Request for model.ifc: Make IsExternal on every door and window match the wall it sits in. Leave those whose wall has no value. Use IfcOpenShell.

First a look at what the model holds.

```python
import ifcopenshell
import ifcopenshell.util.element

model = ifcopenshell.open("model.ifc")
print(model.schema)
seen = {}
for e in model.by_type("IfcDoor") + model.by_type("IfcWindow"):
    if not e.FillsVoids:
        continue
    host = e.FillsVoids[0].RelatingOpeningElement.VoidsElements[0].RelatingBuildingElement
    own = ifcopenshell.util.element.get_pset(e, f"Pset_{e.is_a()[3:].removesuffix('StandardCase')}Common", "IsExternal")
    wall = ifcopenshell.util.element.get_pset(host, "Pset_WallCommon", "IsExternal")
    seen[e.is_a(), own, wall] = seen.get((e.is_a(), own, wall), 0) + 1
for (cls, own, wall), count in sorted(seen.items(), key=str):
    print(count, cls, "IsExternal:", own, "| host wall:", wall)
```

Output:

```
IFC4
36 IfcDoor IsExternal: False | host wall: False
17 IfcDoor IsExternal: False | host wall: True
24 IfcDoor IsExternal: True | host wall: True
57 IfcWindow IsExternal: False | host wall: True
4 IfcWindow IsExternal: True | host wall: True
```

```python
import ifcopenshell
import ifcopenshell.api.pset
import ifcopenshell.util.element

model = ifcopenshell.open("model.ifc")

count = 0
for ifc_class, pset_name in (("IfcDoor", "Pset_DoorCommon"), ("IfcWindow", "Pset_WindowCommon")):
    for e in model.by_type(ifc_class):
        if not e.FillsVoids:
            continue
        host = e.FillsVoids[0].RelatingOpeningElement.VoidsElements[0].RelatingBuildingElement
        external = ifcopenshell.util.element.get_pset(host, "Pset_WallCommon", "IsExternal")
        if external is None or ifcopenshell.util.element.get_pset(e, pset_name, "IsExternal") == external:
            continue
        pset = ifcopenshell.api.pset.add_pset(model, product=e, name=pset_name)
        ifcopenshell.api.pset.edit_pset(model, pset=pset, properties={"IsExternal": external})
        count += 1

print(count, "updated")

model.write("model_edited.ifc")
```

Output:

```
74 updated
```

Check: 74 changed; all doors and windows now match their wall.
